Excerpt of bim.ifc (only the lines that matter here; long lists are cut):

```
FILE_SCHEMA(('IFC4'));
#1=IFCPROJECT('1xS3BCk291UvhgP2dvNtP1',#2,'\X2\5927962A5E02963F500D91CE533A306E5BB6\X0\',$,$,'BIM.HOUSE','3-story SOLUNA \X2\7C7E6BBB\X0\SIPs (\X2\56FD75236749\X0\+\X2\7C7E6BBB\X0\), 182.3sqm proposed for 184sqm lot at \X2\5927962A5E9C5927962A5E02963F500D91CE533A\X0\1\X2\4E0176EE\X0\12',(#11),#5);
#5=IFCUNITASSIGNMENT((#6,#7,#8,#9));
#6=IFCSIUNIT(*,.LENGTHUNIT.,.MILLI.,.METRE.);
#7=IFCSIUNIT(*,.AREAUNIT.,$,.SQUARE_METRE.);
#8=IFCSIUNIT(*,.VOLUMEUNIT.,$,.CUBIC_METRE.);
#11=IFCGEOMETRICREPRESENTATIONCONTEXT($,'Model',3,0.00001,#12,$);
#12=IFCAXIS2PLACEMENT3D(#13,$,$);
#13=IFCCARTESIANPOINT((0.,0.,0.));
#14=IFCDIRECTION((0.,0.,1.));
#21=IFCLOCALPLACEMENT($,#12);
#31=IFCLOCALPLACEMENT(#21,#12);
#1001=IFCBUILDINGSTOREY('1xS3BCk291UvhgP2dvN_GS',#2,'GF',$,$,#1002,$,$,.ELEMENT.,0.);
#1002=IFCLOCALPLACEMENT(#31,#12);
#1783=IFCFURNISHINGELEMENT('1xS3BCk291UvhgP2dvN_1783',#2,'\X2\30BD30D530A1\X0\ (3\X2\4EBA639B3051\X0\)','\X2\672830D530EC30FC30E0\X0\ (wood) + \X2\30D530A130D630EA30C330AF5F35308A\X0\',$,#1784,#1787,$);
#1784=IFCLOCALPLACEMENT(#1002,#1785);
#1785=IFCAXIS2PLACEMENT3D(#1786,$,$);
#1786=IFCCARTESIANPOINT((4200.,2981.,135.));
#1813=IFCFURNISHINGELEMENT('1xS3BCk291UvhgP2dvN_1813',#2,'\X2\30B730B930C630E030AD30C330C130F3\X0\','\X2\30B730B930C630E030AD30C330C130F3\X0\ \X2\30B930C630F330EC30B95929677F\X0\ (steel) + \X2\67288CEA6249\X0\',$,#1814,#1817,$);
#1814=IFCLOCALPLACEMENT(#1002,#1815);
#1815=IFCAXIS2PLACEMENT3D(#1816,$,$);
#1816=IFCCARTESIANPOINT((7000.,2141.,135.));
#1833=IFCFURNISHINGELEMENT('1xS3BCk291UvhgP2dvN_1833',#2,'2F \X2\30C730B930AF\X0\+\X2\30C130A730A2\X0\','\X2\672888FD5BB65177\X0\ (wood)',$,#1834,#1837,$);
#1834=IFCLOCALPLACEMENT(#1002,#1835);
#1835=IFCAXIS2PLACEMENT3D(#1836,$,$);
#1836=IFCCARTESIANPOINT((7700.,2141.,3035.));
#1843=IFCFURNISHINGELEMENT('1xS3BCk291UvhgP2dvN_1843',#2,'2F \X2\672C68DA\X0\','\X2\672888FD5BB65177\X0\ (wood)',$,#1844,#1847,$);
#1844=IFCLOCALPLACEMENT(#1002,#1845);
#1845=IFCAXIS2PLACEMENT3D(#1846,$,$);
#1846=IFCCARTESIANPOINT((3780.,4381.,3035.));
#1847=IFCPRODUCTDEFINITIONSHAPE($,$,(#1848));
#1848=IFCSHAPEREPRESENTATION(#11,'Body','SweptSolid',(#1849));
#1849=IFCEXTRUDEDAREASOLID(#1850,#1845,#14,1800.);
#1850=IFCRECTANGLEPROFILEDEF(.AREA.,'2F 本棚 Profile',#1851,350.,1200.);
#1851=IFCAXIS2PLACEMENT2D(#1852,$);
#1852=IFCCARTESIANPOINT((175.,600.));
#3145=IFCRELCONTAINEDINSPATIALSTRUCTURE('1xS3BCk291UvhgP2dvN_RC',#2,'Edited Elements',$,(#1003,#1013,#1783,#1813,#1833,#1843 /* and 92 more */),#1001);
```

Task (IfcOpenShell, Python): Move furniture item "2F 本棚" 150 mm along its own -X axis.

```python
import ifcopenshell
import ifcopenshell.api.geometry
import ifcopenshell.util.placement
import ifcopenshell.util.unit

model = ifcopenshell.open("bim.ifc")
unit_scale = ifcopenshell.util.unit.calculate_unit_scale(model)

item = model.by_id(1843)
matrix = ifcopenshell.util.placement.get_local_placement(item.ObjectPlacement)
matrix[:3, 3] -= matrix[:3, 0] * 0.15 / unit_scale
ifcopenshell.api.geometry.edit_object_placement(model, product=item, matrix=matrix, is_si=False)

print(ifcopenshell.util.placement.get_local_placement(item.ObjectPlacement).round(3) + 0.0)

model.write("bim_edited.ifc")
```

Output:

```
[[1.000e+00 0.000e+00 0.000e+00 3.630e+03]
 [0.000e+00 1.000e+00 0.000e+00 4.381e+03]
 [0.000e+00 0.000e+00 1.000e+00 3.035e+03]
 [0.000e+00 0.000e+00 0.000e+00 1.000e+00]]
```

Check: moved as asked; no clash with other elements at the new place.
